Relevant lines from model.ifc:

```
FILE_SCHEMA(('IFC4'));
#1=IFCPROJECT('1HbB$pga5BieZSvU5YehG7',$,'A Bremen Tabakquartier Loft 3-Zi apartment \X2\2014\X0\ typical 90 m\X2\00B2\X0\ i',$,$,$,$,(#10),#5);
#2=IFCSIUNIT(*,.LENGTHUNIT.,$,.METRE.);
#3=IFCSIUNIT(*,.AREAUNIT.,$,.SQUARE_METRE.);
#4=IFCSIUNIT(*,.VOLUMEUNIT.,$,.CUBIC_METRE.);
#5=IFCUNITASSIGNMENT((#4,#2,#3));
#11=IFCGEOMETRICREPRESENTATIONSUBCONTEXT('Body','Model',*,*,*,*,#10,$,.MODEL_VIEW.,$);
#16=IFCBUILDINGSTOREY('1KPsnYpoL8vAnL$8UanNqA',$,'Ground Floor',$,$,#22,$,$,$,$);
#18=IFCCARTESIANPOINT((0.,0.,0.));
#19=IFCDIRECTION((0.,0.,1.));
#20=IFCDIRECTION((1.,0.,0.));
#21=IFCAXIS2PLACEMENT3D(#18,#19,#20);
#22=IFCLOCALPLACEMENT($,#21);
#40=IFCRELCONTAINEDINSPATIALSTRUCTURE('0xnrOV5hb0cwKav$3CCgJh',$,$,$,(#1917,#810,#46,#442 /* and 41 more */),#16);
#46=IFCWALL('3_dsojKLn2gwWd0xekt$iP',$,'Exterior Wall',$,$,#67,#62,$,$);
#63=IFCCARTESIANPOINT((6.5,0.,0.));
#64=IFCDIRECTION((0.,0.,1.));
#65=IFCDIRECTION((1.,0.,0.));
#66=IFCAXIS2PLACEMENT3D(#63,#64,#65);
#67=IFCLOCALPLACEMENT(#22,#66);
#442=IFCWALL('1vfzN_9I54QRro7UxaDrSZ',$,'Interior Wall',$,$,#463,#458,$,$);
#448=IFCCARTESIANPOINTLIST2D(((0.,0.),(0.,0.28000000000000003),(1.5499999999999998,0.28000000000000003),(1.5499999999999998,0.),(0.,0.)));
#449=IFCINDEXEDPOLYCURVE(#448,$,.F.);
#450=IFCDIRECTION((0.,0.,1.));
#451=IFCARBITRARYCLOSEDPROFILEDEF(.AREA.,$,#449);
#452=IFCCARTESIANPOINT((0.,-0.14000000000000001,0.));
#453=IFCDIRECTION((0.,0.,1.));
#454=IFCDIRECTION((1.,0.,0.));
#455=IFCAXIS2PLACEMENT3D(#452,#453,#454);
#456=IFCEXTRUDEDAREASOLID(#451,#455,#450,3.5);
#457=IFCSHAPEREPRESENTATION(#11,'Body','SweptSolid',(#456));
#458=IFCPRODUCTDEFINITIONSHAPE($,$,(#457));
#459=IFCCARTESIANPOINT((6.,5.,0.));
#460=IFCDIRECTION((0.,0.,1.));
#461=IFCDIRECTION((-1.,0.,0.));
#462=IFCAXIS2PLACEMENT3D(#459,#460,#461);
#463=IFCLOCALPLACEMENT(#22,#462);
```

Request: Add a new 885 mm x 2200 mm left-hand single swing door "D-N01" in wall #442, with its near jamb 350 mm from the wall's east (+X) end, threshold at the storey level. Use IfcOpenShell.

```python
import numpy as np
import ifcopenshell
import ifcopenshell.api.feature
import ifcopenshell.api.geometry
import ifcopenshell.api.root
import ifcopenshell.api.spatial
import ifcopenshell.geom
import ifcopenshell.util.element
import ifcopenshell.util.placement
import ifcopenshell.util.representation
import ifcopenshell.util.shape
import ifcopenshell.util.unit

model = ifcopenshell.open("model.ifc")
unit_scale = ifcopenshell.util.unit.calculate_unit_scale(model)
settings = ifcopenshell.geom.settings()


def volume(element):
    """Net volume in cubic metres, openings subtracted."""
    shape = ifcopenshell.geom.create_shape(settings, element)
    return ifcopenshell.util.shape.get_volume(shape.geometry)


wall = model.by_guid("1vfzN_9I54QRro7UxaDrSZ")
storey = ifcopenshell.util.element.get_container(wall, ifc_class="IfcBuildingStorey")
context = ifcopenshell.util.representation.get_context(model, "Model", "Body", "MODEL_VIEW")
before = volume(wall)

width, height, from_end, sill = 0.885, 2.2, 0.35, 0.0  # metres

# The wall runs along its own X axis, and the end named is its -X end.
wall_shape = ifcopenshell.geom.create_shape(settings, wall)
x, y, z = ifcopenshell.util.shape.get_vertices(wall_shape.geometry).T
start = x.min() + from_end
face, thickness = float(y.min()), float(y.max() - y.min())
wall_matrix = ifcopenshell.util.placement.get_local_placement(wall.ObjectPlacement)
level = ifcopenshell.util.placement.get_local_placement(storey.ObjectPlacement)[2, 3]


def in_wall(x, y):
    """Placement at x, y metres in the wall's axes, at sill height."""
    matrix = wall_matrix.copy()
    matrix[:, 3] = wall_matrix @ np.array([x / unit_scale, y / unit_scale, 0.0, 1.0])
    matrix[2, 3] = level + sill / unit_scale
    return matrix


# Opening: a box that overshoots both wall faces by 50 mm.
opening = ifcopenshell.api.root.create_entity(model, ifc_class="IfcOpeningElement", predefined_type="OPENING")
box = ifcopenshell.api.geometry.add_wall_representation(
    model, context=context, length=width, height=height, thickness=thickness + 0.1
)
ifcopenshell.api.geometry.assign_representation(model, product=opening, representation=box)
ifcopenshell.api.geometry.edit_object_placement(model, product=opening, matrix=in_wall(start, face - 0.05), is_si=False)
ifcopenshell.api.feature.add_feature(model, feature=opening, element=wall)

door = ifcopenshell.api.root.create_entity(model, ifc_class="IfcDoor", name="D-N01", predefined_type="DOOR")
door.OverallWidth, door.OverallHeight = width / unit_scale, height / unit_scale
door.OperationType = "SINGLE_SWING_LEFT"
body = ifcopenshell.api.geometry.add_door_representation(
    model,
    context=context,
    overall_width=door.OverallWidth,
    overall_height=door.OverallHeight,
    operation_type="SINGLE_SWING_LEFT",
    lining_properties={"LiningDepth": thickness / unit_scale, "ThresholdDepth": thickness / unit_scale},
)
ifcopenshell.api.geometry.assign_representation(model, product=door, representation=body)
ifcopenshell.api.spatial.assign_container(model, products=[door], relating_structure=storey)
ifcopenshell.api.feature.add_filling(model, opening=opening, element=door)

# The lining spans the wall, so the door starts at the wall face.
ifcopenshell.api.geometry.edit_object_placement(model, product=door, matrix=in_wall(start, face), is_si=False)

after = volume(wall)

print(f"wall volume {before:.3f} -> {after:.3f} m3")

model.write("model_v2.ifc")
```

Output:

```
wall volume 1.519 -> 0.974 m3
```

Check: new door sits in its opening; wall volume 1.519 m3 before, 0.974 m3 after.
